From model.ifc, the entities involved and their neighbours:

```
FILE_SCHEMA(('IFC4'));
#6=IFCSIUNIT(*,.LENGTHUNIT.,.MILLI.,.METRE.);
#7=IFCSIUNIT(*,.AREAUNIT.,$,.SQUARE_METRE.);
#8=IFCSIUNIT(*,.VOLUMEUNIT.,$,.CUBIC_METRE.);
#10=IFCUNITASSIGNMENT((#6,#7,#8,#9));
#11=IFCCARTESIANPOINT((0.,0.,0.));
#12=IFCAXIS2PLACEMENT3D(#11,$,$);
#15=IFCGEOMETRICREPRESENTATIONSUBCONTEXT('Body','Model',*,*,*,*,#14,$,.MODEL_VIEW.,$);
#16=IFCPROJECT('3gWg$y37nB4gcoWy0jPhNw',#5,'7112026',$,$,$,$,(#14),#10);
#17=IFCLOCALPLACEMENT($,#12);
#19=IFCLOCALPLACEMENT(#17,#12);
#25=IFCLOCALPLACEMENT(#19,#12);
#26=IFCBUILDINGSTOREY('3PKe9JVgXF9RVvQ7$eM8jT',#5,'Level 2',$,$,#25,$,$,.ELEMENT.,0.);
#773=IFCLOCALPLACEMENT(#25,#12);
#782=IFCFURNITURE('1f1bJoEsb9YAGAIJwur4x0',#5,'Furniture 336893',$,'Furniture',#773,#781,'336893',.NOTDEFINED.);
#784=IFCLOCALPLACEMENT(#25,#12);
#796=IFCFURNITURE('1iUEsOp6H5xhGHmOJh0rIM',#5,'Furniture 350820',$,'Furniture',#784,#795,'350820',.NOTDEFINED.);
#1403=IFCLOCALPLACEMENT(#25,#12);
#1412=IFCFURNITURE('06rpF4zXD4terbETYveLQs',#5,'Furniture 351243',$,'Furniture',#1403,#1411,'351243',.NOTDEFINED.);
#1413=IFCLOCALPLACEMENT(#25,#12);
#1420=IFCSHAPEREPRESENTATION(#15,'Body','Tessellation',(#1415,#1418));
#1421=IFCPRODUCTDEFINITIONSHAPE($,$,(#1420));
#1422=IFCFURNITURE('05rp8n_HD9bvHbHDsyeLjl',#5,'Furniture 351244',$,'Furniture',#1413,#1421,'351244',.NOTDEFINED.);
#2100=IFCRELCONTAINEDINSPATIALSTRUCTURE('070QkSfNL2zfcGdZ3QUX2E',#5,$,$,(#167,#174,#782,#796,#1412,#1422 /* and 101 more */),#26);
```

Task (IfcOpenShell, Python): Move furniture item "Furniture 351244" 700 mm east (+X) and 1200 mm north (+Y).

```python
import ifcopenshell
import ifcopenshell.api.geometry
import ifcopenshell.util.placement
import ifcopenshell.util.unit

model = ifcopenshell.open("model.ifc")
unit_scale = ifcopenshell.util.unit.calculate_unit_scale(model)

item = model.by_guid("05rp8n_HD9bvHbHDsyeLjl")
matrix = ifcopenshell.util.placement.get_local_placement(item.ObjectPlacement)
matrix[0, 3] += 0.7 / unit_scale
matrix[1, 3] += 1.2 / unit_scale
ifcopenshell.api.geometry.edit_object_placement(model, product=item, matrix=matrix, is_si=False)

print(ifcopenshell.util.placement.get_local_placement(item.ObjectPlacement).round(3) + 0.0)

model.write("model_rev.ifc")
```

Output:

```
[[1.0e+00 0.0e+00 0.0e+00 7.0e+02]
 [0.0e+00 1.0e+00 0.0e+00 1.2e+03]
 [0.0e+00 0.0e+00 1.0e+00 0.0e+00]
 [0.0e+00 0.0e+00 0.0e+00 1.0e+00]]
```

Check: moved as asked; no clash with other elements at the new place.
